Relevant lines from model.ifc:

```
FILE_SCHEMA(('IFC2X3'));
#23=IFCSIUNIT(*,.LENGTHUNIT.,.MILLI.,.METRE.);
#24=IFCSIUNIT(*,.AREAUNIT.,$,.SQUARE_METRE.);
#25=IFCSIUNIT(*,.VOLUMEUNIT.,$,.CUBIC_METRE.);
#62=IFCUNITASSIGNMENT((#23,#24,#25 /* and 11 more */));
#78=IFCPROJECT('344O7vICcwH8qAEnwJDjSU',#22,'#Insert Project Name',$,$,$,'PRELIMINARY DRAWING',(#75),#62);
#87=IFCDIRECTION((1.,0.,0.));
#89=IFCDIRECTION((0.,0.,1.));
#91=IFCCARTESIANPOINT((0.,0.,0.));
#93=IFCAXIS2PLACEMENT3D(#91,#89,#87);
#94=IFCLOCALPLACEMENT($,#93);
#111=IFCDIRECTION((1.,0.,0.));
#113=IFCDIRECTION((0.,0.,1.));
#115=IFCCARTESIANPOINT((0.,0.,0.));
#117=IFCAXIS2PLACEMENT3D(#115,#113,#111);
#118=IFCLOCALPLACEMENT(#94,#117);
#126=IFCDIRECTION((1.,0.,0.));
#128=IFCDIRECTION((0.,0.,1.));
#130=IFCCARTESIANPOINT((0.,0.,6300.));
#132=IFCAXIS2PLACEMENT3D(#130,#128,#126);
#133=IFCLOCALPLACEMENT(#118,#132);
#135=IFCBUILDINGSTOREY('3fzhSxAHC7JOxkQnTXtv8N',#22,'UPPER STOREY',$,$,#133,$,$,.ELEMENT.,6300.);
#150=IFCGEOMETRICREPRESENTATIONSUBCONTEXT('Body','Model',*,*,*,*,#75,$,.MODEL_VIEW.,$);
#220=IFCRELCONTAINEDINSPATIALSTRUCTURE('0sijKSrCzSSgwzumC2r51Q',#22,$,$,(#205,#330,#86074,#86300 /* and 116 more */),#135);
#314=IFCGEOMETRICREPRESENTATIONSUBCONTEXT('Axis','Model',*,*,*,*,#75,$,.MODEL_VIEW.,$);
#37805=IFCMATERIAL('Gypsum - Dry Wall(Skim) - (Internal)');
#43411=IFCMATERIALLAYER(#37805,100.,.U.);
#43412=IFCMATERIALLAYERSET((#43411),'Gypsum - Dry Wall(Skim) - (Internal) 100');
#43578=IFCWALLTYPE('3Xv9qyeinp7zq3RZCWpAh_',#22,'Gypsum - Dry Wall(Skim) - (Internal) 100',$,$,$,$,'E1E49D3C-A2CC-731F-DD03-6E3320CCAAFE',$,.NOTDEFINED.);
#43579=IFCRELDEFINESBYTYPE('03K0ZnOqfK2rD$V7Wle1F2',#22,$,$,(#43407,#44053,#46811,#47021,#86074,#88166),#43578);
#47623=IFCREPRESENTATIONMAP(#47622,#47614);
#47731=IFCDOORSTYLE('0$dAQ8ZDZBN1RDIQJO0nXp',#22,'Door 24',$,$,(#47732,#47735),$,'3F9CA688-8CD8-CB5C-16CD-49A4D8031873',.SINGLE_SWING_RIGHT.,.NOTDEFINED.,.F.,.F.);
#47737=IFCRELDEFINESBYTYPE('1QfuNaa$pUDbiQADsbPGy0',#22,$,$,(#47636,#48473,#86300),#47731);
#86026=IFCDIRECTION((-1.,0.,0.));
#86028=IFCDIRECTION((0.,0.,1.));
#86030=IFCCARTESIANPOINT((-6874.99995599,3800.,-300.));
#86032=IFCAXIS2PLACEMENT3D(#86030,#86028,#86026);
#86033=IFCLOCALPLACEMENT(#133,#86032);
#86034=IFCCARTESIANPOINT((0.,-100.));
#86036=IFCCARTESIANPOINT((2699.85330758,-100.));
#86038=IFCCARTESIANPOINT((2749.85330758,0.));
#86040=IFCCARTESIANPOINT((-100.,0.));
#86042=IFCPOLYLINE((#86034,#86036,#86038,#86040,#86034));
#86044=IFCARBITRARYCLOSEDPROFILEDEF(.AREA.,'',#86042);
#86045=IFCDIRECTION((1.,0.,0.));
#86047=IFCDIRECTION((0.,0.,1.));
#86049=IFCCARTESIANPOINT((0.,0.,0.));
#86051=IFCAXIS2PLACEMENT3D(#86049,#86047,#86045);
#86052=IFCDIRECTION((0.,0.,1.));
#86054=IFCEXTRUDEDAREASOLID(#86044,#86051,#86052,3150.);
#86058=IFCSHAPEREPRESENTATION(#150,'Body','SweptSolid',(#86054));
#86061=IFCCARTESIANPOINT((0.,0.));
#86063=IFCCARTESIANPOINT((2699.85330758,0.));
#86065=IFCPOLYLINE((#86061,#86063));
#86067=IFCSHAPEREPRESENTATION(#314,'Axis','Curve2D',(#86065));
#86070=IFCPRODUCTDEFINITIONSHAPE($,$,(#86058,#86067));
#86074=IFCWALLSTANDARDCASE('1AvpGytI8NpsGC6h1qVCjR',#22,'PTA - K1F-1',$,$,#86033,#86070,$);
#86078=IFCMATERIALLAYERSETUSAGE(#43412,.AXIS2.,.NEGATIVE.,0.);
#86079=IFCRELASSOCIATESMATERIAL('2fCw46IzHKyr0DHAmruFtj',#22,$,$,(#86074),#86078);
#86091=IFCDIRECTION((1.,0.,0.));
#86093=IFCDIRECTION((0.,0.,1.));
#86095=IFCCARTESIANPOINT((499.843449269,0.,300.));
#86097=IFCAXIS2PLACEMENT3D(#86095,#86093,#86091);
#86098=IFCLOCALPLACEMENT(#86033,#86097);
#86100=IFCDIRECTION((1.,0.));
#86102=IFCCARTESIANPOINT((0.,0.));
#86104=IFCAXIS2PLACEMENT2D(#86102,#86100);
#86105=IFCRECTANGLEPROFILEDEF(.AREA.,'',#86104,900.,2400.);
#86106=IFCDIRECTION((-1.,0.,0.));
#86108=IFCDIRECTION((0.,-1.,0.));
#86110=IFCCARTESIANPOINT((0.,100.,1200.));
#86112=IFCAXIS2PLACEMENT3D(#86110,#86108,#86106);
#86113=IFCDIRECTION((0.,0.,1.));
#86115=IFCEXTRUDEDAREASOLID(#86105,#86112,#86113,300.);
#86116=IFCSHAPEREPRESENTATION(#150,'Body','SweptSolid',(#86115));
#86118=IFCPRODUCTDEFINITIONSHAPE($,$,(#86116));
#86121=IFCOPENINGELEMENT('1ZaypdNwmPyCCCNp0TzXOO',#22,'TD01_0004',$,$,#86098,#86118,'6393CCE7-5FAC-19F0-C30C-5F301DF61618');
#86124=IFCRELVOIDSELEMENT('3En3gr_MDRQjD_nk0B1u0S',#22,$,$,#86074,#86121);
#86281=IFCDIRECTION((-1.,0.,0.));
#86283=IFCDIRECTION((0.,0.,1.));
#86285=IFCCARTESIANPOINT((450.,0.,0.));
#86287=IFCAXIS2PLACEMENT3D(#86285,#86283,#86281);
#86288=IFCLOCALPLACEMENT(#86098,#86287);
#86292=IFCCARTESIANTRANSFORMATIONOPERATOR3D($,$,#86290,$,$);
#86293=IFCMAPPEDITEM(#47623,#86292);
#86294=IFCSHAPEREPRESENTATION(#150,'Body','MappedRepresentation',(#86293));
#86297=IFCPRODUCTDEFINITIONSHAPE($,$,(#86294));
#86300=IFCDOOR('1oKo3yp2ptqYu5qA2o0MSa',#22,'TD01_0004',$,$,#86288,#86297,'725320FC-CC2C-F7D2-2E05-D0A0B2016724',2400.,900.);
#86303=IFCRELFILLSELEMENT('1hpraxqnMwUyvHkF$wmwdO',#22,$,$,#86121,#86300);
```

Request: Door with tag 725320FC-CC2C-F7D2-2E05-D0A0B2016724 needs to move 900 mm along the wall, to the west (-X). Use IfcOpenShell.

```python
import ifcopenshell
import ifcopenshell.api.geometry
import ifcopenshell.util.placement
import ifcopenshell.util.unit

model = ifcopenshell.open("model.ifc")
unit_scale = ifcopenshell.util.unit.calculate_unit_scale(model)

door = model.by_guid("1oKo3yp2ptqYu5qA2o0MSa")
opening = door.FillsVoids[0].RelatingOpeningElement
wall = opening.VoidsElements[0].RelatingBuildingElement

wall_matrix = ifcopenshell.util.placement.get_local_placement(wall.ObjectPlacement)
shift = wall_matrix[:3, 0] * 0.9 / unit_scale
before = ifcopenshell.util.placement.get_local_placement(door.ObjectPlacement)[:3, 3].copy()

# The door is placed relative to its opening, so it follows when the opening moves.
matrix = ifcopenshell.util.placement.get_local_placement(opening.ObjectPlacement)
matrix[:3, 3] += shift
ifcopenshell.api.geometry.edit_object_placement(
    model, product=opening, matrix=matrix, is_si=False, should_transform_children=True
)

after = ifcopenshell.util.placement.get_local_placement(door.ObjectPlacement)[:3, 3]
print("door moved by", (after - before).round(3) + 0.0)

model.write("model_edited.ifc")
```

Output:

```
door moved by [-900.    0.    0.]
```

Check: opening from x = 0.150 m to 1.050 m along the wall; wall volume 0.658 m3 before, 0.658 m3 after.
